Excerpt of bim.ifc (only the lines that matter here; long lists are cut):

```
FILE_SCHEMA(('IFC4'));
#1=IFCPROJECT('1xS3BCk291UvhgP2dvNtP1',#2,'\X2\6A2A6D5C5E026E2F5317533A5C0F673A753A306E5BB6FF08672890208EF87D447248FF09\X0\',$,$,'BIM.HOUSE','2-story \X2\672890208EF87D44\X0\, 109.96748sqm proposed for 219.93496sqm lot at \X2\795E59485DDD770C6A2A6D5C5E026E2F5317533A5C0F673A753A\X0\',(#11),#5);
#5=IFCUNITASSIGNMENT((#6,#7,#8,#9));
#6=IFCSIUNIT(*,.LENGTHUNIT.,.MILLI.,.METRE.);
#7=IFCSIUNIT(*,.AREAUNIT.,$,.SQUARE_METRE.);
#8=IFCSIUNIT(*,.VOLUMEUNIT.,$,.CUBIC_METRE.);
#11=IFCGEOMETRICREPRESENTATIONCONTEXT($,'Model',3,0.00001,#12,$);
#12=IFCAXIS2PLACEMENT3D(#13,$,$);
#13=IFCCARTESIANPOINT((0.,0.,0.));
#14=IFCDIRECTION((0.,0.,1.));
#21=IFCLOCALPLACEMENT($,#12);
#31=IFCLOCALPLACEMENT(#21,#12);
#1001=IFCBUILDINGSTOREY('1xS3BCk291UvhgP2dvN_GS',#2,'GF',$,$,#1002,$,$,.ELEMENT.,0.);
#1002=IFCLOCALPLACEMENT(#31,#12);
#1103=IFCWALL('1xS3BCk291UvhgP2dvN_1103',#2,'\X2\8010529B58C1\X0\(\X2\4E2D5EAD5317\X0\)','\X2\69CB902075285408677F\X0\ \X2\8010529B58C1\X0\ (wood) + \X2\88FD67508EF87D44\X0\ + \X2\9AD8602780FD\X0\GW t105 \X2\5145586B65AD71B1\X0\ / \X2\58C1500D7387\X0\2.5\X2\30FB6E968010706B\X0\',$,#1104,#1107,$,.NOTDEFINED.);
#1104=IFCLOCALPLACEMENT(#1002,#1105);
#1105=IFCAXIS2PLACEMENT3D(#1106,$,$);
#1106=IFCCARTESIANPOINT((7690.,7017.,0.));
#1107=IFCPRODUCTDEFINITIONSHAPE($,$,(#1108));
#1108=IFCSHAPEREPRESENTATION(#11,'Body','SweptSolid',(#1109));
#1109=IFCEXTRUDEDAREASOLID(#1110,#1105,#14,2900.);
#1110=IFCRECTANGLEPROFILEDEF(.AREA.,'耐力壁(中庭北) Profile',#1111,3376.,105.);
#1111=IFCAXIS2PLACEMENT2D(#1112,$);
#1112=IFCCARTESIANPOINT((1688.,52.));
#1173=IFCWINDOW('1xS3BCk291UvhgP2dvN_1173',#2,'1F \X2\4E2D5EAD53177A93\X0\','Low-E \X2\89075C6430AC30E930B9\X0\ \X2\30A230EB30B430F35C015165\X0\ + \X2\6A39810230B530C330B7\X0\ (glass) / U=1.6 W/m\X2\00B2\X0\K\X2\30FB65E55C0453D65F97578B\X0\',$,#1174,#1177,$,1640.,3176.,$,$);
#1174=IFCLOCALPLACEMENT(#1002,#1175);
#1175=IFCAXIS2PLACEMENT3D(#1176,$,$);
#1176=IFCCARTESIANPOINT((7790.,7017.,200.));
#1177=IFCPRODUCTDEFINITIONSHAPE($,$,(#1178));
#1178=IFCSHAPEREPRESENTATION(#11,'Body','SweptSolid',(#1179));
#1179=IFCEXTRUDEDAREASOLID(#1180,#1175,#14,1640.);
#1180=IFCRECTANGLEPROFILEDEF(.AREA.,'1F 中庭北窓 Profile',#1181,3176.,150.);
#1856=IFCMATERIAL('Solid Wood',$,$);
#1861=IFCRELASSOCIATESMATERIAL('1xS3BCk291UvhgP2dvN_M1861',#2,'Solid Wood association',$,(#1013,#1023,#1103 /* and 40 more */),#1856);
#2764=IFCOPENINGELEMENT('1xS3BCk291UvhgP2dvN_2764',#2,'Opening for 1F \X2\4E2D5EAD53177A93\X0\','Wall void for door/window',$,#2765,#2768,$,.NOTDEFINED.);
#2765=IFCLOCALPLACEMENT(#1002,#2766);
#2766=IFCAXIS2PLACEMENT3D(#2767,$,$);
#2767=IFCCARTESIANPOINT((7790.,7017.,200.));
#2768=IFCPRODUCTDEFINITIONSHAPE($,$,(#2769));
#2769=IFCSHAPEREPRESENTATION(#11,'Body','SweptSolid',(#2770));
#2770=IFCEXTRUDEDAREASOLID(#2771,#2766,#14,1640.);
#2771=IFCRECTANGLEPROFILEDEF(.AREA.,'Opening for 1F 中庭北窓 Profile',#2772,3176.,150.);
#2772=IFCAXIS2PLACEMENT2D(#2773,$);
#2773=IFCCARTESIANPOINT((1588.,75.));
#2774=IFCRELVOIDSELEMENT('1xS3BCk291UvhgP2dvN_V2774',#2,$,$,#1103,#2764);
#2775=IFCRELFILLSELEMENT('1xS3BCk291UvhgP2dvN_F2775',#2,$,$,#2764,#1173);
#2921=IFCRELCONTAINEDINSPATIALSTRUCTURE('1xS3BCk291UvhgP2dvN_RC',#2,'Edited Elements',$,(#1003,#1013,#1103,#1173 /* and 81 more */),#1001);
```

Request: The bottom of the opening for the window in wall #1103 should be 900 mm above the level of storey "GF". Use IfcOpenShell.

```python
import numpy as np
import ifcopenshell
import ifcopenshell.api.geometry
import ifcopenshell.geom
import ifcopenshell.util.element
import ifcopenshell.util.placement
import ifcopenshell.util.shape
import ifcopenshell.util.unit

model = ifcopenshell.open("bim.ifc")
unit_scale = ifcopenshell.util.unit.calculate_unit_scale(model)

window = model.by_id(1173)
opening = window.FillsVoids[0].RelatingOpeningElement
storey = ifcopenshell.util.element.get_container(window, ifc_class="IfcBuildingStorey")
level = ifcopenshell.util.placement.get_local_placement(storey.ObjectPlacement)[2, 3]

# The opening's origin need not be at the sill, so measure its lowest point.
shape = ifcopenshell.geom.create_shape(ifcopenshell.geom.settings(), opening)
bottom = ifcopenshell.util.shape.get_shape_bottom_elevation(shape, shape.geometry) / unit_scale
dz = level + 0.9 / unit_scale - bottom

shift = np.array([0.0, 0.0, dz])
# The window is not placed relative to its opening, so move both.
for product in (opening, window):
    matrix = ifcopenshell.util.placement.get_local_placement(product.ObjectPlacement)
    matrix[:3, 3] += shift
    ifcopenshell.api.geometry.edit_object_placement(model, product=product, matrix=matrix, is_si=False)

print(f"moved by {dz * unit_scale:+.3f} m")

model.write("bim-out.ifc")
```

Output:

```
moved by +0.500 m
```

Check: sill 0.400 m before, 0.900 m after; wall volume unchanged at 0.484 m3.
